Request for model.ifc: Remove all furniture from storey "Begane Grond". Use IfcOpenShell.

First a look at what the model holds.

```python
import ifcopenshell
import ifcopenshell.util.element

model = ifcopenshell.open("model.ifc")
print(model.schema)
storey = next(s for s in model.by_type("IfcBuildingStorey") if s.Name == "Begane Grond")
furniture = [e for e in ifcopenshell.util.element.get_decomposition(storey) if e.is_a("IfcFurnishingElement")]
seen = {}
for e in furniture:
    element_type = ifcopenshell.util.element.get_type(e)
    name = element_type.Name if element_type not in (None, e) else None
    seen[name] = seen.get(name, 0) + 1
for name, count in sorted(seen.items(), key=str):
    print(count, "x", name)
```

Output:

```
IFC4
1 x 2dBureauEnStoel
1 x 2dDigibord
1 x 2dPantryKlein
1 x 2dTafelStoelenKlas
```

```python
import ifcopenshell
import ifcopenshell.api.root
import ifcopenshell.util.element

model = ifcopenshell.open("model.ifc")

storey = next(s for s in model.by_type("IfcBuildingStorey") if s.Name == "Begane Grond")
furniture = [e for e in ifcopenshell.util.element.get_decomposition(storey) if e.is_a("IfcFurnishingElement")]

for e in furniture:
    ifcopenshell.api.root.remove_product(model, product=e)
print(len(furniture), "removed")

model.write("model_edited.ifc")
```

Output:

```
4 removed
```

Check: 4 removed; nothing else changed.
